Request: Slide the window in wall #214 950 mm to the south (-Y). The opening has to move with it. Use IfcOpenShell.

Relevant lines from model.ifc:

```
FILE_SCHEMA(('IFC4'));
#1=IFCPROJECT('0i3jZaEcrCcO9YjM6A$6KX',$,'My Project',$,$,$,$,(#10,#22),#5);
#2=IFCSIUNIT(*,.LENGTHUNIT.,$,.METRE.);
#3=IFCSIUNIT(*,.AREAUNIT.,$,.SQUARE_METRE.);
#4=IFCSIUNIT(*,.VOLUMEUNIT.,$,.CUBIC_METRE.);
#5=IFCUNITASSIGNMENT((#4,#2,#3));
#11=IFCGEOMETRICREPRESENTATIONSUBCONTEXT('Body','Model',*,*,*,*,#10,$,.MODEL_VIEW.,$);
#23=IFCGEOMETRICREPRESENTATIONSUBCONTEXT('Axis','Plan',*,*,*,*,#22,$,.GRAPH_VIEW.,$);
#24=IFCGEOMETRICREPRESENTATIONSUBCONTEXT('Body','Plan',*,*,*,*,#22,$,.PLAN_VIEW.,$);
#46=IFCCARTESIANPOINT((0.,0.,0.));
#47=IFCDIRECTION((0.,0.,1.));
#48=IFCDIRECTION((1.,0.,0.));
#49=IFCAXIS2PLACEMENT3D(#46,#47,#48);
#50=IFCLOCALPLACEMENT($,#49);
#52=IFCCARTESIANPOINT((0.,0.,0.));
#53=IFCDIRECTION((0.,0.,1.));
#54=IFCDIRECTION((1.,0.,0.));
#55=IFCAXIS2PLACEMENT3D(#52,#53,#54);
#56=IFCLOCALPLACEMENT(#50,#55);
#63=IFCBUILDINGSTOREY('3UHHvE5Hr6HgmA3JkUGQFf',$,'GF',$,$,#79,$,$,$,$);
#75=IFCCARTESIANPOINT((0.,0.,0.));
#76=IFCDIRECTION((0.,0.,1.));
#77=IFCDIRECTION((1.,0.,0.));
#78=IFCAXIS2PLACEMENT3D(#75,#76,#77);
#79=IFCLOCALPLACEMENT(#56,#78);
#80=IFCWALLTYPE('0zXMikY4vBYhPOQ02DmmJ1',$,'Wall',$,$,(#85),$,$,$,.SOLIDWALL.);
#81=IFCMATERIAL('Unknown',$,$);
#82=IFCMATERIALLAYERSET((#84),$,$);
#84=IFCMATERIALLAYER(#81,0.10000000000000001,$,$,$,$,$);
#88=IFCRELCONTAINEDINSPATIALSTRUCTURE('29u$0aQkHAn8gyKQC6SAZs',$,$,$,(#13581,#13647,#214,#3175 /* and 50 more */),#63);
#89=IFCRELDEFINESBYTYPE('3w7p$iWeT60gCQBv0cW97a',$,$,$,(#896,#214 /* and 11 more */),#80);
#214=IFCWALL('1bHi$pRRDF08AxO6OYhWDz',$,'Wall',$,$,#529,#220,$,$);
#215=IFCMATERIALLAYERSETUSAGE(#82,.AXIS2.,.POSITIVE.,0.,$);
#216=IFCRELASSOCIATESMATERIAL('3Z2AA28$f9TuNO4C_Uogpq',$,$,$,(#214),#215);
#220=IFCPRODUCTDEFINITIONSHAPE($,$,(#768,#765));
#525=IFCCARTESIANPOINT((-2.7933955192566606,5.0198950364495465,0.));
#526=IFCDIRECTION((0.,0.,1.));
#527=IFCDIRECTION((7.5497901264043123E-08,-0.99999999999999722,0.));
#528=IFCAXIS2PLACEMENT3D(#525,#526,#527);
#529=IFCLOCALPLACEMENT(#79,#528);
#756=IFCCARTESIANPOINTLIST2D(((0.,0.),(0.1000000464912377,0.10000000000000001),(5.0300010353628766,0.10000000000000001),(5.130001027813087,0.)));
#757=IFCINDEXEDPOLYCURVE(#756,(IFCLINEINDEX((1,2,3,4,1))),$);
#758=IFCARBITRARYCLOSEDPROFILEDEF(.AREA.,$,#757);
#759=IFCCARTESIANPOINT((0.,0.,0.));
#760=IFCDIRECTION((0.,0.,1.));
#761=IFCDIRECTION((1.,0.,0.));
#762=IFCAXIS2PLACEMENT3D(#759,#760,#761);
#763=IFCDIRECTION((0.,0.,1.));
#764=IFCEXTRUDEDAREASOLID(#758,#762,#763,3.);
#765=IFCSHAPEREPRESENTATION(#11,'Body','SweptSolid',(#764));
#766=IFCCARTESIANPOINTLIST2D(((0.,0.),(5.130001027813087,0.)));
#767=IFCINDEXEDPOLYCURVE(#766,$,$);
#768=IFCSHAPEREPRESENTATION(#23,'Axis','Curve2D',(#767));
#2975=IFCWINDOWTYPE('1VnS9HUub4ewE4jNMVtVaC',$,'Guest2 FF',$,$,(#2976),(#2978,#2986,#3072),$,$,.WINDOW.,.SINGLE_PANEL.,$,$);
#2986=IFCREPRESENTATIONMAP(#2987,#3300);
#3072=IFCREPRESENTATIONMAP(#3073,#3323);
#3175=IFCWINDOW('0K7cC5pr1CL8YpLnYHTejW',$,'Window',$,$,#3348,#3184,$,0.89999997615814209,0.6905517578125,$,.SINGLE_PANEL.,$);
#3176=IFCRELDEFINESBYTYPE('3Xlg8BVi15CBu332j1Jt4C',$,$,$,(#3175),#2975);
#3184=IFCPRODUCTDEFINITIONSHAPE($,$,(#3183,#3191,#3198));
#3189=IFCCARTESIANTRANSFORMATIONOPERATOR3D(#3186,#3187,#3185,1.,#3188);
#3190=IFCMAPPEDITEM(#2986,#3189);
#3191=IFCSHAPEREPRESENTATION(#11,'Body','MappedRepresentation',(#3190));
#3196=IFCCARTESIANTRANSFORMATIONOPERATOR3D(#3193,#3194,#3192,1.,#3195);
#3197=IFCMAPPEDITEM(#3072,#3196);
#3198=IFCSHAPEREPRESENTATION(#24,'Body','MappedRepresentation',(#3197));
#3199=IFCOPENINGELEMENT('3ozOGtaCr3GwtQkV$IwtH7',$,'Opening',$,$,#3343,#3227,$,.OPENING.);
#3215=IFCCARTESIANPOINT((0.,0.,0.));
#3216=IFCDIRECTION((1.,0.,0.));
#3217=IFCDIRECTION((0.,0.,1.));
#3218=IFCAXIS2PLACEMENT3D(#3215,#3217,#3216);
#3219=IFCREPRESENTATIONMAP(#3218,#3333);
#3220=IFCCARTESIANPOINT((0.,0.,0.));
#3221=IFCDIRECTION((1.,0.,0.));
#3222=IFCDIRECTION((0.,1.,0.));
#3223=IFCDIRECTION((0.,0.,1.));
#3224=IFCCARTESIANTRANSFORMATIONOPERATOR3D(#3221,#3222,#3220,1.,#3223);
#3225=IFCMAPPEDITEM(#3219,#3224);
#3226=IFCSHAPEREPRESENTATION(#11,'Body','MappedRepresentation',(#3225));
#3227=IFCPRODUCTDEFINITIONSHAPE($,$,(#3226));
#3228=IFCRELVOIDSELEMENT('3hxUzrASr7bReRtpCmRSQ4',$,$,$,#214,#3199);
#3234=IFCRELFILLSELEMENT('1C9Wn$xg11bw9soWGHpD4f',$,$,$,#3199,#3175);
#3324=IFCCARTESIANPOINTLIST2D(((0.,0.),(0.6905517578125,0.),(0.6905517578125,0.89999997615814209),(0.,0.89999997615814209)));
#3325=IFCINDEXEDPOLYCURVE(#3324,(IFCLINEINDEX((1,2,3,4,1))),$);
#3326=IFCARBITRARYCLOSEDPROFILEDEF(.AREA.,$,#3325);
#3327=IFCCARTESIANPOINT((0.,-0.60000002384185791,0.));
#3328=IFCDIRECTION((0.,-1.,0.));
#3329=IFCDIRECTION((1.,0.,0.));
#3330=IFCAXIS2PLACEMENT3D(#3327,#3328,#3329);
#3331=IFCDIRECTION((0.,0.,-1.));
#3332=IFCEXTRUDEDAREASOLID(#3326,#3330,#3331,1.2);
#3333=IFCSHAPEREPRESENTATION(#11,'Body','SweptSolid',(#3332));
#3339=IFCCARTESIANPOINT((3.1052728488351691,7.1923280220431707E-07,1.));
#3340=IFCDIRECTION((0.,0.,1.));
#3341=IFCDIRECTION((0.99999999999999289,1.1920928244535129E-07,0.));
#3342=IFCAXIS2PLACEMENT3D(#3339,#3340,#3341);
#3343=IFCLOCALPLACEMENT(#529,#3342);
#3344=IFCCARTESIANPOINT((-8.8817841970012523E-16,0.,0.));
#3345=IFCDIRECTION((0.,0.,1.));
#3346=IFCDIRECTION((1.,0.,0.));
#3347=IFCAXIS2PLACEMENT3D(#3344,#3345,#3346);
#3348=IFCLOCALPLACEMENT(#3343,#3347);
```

```python
import ifcopenshell
import ifcopenshell.api.geometry
import ifcopenshell.util.placement

model = ifcopenshell.open("model.ifc")

window = model.by_guid("0K7cC5pr1CL8YpLnYHTejW")
opening = window.FillsVoids[0].RelatingOpeningElement
wall = opening.VoidsElements[0].RelatingBuildingElement

wall_matrix = ifcopenshell.util.placement.get_local_placement(wall.ObjectPlacement)
shift = wall_matrix[:3, 0] * 0.95
before = ifcopenshell.util.placement.get_local_placement(window.ObjectPlacement)[:3, 3].copy()

# The window is placed relative to its opening, so it follows when the opening moves.
matrix = ifcopenshell.util.placement.get_local_placement(opening.ObjectPlacement)
matrix[:3, 3] += shift
ifcopenshell.api.geometry.edit_object_placement(
    model, product=opening, matrix=matrix, is_si=False, should_transform_children=True
)

after = ifcopenshell.util.placement.get_local_placement(window.ObjectPlacement)[:3, 3]
print("window moved by", (after - before).round(3) + 0.0)

model.write("model_v2.ifc")
```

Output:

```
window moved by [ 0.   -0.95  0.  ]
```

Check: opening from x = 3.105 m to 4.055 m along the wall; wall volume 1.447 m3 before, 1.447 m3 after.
